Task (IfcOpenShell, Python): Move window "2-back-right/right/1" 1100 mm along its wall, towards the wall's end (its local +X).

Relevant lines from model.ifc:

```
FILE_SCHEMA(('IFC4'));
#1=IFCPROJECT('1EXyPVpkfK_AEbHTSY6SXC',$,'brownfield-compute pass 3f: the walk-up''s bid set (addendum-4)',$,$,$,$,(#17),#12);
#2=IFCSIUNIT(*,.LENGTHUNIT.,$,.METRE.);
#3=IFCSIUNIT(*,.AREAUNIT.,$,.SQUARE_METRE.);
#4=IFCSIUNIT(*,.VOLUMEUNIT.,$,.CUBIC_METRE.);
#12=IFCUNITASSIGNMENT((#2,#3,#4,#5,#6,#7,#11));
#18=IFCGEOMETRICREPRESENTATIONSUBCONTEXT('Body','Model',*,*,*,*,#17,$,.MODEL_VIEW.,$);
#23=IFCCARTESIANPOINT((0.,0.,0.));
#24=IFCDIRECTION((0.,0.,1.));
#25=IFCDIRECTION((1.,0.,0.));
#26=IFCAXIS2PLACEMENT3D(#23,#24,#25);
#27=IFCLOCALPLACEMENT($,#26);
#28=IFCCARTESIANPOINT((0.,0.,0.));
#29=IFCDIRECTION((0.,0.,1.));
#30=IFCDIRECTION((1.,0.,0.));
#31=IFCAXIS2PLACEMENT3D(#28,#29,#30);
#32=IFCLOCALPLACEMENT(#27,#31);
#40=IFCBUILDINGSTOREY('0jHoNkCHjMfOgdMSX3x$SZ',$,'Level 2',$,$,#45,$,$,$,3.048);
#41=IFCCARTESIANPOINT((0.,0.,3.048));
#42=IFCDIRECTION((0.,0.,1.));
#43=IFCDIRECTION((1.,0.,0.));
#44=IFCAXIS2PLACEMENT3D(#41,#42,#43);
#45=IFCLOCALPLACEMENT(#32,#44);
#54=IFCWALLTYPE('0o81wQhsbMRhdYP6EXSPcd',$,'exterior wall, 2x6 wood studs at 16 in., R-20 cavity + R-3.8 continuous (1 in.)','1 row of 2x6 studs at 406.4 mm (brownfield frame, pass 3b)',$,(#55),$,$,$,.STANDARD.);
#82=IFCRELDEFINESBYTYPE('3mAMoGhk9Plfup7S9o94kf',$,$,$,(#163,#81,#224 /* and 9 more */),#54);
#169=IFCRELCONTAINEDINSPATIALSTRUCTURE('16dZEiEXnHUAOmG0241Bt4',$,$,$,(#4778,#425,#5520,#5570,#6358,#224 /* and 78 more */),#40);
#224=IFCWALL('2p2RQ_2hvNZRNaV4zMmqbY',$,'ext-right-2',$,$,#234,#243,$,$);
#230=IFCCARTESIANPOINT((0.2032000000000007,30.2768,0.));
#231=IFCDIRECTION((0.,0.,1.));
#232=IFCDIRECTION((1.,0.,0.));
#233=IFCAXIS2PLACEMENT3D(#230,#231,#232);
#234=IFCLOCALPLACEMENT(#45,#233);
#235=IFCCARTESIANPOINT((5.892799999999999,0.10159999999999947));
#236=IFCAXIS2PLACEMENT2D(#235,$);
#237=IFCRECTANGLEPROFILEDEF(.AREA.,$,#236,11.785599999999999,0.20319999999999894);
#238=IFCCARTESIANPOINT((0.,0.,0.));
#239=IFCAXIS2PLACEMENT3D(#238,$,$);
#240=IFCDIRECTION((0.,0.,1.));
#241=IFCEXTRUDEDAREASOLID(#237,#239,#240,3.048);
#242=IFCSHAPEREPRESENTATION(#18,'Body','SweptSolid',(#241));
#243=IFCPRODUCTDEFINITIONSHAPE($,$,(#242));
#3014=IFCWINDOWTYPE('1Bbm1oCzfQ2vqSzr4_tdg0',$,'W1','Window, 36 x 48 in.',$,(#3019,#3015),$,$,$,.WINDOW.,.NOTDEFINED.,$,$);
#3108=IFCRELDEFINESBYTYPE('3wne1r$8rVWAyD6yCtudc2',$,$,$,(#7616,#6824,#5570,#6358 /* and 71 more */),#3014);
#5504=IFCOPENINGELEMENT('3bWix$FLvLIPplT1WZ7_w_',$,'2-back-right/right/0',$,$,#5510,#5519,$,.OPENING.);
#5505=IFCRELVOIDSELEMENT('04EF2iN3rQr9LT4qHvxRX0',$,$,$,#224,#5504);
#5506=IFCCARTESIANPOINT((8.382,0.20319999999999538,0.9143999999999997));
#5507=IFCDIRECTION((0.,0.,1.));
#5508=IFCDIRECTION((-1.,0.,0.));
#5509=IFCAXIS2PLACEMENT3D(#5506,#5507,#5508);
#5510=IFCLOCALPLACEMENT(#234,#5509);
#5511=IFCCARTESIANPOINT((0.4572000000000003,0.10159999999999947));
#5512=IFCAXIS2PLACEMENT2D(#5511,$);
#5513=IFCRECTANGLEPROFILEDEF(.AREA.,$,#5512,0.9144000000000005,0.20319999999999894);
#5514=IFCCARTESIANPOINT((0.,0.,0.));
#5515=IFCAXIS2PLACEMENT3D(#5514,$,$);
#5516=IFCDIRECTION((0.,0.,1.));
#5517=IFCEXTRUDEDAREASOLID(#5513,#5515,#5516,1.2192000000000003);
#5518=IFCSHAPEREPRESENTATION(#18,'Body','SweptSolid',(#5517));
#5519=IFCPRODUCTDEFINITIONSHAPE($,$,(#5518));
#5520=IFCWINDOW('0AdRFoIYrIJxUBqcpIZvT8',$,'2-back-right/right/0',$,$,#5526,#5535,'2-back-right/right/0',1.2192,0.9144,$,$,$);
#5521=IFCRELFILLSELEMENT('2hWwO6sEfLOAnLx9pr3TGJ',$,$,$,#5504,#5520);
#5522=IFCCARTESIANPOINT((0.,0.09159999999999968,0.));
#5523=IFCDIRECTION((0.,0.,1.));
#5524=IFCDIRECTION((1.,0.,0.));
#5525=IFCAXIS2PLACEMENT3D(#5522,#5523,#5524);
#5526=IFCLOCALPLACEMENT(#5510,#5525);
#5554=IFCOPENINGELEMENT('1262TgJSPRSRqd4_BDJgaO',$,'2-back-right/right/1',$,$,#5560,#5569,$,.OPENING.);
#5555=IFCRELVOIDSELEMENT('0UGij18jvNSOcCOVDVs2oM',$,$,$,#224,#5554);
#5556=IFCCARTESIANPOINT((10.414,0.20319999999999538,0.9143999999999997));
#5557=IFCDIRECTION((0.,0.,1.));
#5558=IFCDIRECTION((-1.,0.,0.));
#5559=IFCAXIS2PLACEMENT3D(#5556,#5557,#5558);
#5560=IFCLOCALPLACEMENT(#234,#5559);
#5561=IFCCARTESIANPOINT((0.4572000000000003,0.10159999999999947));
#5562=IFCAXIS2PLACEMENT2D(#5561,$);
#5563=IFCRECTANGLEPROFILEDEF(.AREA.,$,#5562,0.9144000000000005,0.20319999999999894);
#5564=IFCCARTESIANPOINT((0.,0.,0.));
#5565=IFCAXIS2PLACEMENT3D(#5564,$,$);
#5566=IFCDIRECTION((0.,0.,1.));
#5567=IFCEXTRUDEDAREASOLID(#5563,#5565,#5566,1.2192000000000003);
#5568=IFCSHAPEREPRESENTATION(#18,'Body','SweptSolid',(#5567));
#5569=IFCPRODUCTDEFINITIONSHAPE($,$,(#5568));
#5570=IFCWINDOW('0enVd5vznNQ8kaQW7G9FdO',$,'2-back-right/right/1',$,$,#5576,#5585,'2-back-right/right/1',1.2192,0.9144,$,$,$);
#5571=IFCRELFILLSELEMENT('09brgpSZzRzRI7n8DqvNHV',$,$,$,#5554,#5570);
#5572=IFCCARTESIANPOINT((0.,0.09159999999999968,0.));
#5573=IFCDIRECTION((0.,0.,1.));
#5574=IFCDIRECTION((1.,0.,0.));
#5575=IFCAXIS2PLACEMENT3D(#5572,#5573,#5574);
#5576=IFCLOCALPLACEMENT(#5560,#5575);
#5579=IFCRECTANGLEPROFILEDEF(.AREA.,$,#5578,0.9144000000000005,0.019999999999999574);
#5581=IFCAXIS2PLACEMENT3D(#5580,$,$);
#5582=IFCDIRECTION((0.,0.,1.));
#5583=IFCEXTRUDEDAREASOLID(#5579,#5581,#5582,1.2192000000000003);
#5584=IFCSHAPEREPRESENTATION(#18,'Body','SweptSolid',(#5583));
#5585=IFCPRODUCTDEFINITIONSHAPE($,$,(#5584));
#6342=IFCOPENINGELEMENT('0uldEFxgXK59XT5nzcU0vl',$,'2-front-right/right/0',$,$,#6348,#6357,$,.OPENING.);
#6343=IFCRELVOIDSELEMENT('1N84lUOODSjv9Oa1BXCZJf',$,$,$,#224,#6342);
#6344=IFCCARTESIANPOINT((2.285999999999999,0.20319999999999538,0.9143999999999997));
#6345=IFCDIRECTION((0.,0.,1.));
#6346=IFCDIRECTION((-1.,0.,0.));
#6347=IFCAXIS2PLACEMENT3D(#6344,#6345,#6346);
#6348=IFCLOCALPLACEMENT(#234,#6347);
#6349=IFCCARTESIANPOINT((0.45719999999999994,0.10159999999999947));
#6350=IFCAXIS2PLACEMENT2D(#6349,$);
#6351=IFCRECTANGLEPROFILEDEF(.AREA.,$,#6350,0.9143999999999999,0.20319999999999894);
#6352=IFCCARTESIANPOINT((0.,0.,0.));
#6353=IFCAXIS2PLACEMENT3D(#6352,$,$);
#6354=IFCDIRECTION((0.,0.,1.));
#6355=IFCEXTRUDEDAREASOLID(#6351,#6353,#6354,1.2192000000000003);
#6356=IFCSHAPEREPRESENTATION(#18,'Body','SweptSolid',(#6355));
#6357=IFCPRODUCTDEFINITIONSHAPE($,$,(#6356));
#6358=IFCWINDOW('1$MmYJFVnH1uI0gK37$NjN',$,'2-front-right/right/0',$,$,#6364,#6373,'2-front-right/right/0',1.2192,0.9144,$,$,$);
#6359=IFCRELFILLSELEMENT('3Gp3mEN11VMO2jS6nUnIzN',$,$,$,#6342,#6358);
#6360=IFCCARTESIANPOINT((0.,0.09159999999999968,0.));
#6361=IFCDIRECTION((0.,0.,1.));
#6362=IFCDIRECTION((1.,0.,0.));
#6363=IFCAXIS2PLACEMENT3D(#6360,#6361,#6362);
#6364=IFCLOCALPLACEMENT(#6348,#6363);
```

```python
import ifcopenshell
import ifcopenshell.api.geometry
import ifcopenshell.util.placement
import ifcopenshell.util.unit

model = ifcopenshell.open("model.ifc")
unit_scale = ifcopenshell.util.unit.calculate_unit_scale(model)

window = model.by_guid("0enVd5vznNQ8kaQW7G9FdO")
opening = window.FillsVoids[0].RelatingOpeningElement
wall = opening.VoidsElements[0].RelatingBuildingElement

wall_matrix = ifcopenshell.util.placement.get_local_placement(wall.ObjectPlacement)
shift = wall_matrix[:3, 0] * 1.1 / unit_scale
before = ifcopenshell.util.placement.get_local_placement(window.ObjectPlacement)[:3, 3].copy()

# The window is placed relative to its opening, so it follows when the opening moves.
matrix = ifcopenshell.util.placement.get_local_placement(opening.ObjectPlacement)
matrix[:3, 3] += shift
ifcopenshell.api.geometry.edit_object_placement(
    model, product=opening, matrix=matrix, is_si=False, should_transform_children=True
)

after = ifcopenshell.util.placement.get_local_placement(window.ObjectPlacement)[:3, 3]
print("window moved by", (after - before).round(3) + 0.0)

model.write("model_updated.ifc")
```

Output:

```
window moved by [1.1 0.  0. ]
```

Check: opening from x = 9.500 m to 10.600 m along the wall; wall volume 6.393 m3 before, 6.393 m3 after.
